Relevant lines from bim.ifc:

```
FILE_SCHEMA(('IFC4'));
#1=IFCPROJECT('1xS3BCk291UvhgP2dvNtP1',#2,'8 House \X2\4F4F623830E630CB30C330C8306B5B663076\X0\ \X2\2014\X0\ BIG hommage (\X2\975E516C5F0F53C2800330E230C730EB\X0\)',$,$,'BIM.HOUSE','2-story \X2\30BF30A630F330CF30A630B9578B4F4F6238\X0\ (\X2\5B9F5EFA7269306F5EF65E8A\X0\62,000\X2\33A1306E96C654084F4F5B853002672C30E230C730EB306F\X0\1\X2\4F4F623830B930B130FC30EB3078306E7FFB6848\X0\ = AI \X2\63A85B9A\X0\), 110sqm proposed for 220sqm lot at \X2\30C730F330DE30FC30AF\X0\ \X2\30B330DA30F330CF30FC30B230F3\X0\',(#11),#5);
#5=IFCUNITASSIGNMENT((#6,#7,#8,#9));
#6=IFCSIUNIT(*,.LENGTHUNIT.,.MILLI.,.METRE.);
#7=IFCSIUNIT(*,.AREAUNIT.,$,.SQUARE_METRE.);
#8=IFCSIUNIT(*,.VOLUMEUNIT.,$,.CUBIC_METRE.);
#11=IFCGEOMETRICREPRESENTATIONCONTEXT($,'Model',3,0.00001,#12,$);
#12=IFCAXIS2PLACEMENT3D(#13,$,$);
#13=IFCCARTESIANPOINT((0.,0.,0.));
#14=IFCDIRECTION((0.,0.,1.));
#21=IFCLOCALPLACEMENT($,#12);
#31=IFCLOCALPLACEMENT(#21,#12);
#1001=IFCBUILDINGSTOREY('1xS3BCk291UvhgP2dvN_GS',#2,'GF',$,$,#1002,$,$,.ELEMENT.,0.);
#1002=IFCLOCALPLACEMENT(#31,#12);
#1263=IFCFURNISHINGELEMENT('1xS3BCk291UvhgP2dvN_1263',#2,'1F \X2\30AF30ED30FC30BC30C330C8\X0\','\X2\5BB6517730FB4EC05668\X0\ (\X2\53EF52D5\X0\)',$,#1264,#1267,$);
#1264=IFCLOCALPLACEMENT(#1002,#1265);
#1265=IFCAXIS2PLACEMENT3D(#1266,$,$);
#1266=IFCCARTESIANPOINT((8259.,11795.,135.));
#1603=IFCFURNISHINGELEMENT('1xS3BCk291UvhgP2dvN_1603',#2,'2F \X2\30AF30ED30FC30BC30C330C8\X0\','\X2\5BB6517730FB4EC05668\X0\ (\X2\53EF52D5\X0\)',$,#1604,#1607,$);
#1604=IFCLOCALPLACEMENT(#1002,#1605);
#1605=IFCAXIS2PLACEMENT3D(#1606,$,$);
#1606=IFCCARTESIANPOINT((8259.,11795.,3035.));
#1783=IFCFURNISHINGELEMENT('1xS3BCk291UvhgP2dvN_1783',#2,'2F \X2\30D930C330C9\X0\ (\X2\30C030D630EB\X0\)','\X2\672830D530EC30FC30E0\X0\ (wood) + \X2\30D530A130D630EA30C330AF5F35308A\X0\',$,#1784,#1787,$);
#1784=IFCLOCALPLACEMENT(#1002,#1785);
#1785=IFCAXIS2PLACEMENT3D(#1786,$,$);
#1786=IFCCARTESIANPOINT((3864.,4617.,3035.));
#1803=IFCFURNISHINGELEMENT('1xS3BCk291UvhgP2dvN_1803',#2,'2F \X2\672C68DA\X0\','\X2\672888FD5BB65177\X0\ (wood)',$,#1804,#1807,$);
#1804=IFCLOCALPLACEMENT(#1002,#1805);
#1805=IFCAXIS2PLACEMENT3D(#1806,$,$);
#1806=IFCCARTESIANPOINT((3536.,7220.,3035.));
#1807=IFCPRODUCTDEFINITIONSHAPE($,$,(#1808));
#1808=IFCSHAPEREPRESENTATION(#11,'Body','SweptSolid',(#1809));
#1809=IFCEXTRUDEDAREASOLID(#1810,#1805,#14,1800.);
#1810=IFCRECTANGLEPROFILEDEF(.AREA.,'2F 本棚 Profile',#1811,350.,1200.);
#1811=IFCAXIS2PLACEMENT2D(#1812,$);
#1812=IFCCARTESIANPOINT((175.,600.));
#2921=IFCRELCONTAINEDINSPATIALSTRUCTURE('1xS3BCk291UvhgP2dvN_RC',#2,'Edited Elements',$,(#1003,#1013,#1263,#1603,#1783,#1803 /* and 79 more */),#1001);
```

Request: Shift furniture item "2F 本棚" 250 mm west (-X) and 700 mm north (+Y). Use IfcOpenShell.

```python
import ifcopenshell
import ifcopenshell.api.geometry
import ifcopenshell.util.placement
import ifcopenshell.util.unit

model = ifcopenshell.open("bim.ifc")
unit_scale = ifcopenshell.util.unit.calculate_unit_scale(model)

item = model.by_guid("1xS3BCk291UvhgP2dvN_1803")
matrix = ifcopenshell.util.placement.get_local_placement(item.ObjectPlacement)
matrix[0, 3] -= 0.25 / unit_scale
matrix[1, 3] += 0.7 / unit_scale
ifcopenshell.api.geometry.edit_object_placement(model, product=item, matrix=matrix, is_si=False)

print(ifcopenshell.util.placement.get_local_placement(item.ObjectPlacement).round(3) + 0.0)

model.write("bim_v2.ifc")
```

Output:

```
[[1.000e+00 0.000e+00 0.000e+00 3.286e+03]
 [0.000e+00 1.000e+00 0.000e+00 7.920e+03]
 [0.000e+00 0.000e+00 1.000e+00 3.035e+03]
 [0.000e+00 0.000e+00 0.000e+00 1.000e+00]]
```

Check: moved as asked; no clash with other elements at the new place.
